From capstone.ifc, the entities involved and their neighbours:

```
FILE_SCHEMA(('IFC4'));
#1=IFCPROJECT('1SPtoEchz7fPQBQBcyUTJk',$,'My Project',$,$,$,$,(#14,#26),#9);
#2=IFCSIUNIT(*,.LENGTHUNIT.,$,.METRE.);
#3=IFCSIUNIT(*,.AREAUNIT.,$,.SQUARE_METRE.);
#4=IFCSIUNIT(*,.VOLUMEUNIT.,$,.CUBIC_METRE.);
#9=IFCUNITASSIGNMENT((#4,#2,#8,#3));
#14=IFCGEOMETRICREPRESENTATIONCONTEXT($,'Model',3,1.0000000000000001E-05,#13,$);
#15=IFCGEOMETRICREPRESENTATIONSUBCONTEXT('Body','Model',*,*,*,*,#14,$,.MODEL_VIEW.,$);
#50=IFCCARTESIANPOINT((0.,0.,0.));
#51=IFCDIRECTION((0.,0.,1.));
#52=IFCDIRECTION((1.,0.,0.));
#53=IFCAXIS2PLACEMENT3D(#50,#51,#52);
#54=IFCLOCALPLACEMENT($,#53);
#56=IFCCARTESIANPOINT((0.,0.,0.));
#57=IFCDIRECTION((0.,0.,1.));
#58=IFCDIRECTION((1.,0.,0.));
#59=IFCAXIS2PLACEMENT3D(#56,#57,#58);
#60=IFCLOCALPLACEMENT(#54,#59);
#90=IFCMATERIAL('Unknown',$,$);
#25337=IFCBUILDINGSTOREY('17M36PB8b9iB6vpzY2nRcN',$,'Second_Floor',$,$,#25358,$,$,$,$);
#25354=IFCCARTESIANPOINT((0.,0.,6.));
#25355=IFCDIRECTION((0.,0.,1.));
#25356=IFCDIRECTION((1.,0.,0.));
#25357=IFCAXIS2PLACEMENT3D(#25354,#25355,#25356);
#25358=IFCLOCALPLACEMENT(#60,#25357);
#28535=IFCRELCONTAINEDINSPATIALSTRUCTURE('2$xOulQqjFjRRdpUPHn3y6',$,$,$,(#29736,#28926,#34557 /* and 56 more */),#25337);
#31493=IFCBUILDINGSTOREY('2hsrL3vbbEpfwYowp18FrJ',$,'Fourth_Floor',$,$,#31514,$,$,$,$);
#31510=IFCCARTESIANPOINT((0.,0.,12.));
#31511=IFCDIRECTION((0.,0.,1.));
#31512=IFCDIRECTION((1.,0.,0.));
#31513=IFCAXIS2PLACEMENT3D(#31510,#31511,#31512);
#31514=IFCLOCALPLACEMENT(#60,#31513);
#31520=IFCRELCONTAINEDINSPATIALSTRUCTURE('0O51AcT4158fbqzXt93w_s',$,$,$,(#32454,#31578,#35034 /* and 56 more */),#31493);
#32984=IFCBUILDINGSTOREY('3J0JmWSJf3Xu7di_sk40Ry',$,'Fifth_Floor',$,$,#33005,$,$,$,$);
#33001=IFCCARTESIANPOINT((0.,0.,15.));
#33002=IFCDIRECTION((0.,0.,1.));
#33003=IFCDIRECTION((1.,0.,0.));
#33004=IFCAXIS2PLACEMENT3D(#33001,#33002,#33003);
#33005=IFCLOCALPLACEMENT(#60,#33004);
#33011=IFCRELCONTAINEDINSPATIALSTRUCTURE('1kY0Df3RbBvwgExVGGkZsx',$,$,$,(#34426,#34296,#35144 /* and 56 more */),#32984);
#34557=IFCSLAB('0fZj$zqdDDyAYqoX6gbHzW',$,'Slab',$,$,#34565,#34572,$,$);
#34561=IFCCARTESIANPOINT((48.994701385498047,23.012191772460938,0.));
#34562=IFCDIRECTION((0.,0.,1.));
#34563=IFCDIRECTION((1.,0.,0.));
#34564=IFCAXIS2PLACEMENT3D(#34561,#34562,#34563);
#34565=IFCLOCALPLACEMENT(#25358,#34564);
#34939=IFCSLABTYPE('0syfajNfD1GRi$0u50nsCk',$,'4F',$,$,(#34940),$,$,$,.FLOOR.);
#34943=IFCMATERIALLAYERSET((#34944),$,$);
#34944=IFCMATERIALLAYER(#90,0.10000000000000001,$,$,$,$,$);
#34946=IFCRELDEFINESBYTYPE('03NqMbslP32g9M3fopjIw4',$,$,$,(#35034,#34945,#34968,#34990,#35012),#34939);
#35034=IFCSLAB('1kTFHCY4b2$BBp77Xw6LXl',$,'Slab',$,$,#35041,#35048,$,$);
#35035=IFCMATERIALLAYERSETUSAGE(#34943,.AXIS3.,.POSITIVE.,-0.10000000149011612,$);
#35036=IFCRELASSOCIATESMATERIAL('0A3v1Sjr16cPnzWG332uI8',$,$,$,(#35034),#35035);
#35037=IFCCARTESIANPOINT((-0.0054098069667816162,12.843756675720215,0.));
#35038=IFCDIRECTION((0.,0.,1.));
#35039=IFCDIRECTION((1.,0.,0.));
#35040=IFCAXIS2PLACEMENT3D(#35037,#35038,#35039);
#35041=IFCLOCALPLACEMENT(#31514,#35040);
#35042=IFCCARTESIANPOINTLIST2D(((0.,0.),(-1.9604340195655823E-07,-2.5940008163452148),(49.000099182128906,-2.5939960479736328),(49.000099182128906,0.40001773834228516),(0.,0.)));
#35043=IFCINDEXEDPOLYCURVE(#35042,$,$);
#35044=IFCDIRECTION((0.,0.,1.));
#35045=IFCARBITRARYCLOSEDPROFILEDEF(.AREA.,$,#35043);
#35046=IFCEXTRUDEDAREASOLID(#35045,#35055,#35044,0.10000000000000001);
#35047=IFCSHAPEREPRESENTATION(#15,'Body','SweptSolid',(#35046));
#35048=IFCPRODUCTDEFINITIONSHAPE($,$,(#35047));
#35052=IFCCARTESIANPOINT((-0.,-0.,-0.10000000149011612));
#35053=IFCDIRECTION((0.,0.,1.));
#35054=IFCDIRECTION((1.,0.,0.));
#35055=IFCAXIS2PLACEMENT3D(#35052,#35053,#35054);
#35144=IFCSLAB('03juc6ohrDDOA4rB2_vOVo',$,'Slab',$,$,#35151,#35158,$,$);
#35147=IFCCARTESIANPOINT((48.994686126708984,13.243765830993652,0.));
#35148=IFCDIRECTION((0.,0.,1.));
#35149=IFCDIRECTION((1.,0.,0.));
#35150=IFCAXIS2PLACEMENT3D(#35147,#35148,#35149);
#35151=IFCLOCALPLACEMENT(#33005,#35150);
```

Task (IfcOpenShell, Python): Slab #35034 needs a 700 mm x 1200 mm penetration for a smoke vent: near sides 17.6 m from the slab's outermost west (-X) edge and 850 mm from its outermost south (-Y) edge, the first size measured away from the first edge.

```python
import numpy as np
import ifcopenshell
import ifcopenshell.api.feature
import ifcopenshell.api.geometry
import ifcopenshell.api.root
import ifcopenshell.geom
import ifcopenshell.util.placement
import ifcopenshell.util.representation
import ifcopenshell.util.shape
import ifcopenshell.util.unit

model = ifcopenshell.open("capstone.ifc")
unit_scale = ifcopenshell.util.unit.calculate_unit_scale(model)
settings = ifcopenshell.geom.settings()


def volume(element):
    """Net volume in cubic metres, openings subtracted."""
    shape = ifcopenshell.geom.create_shape(settings, element)
    return ifcopenshell.util.shape.get_volume(shape.geometry)


slab = model.by_guid("1kTFHCY4b2$BBp77Xw6LXl")
before = volume(slab)

# Extent in the slab's own axes, in metres. The edges named are its -X and -Y sides.
slab_shape = ifcopenshell.geom.create_shape(settings, slab)
vertices = ifcopenshell.util.shape.get_vertices(slab_shape.geometry)
x_min, y_min, bottom = vertices.min(axis=0)
top = vertices[:, 2].max()

opening = ifcopenshell.api.root.create_entity(model, ifc_class="IfcOpeningElement", name="Smoke vent opening", predefined_type="OPENING")
context = ifcopenshell.util.representation.get_context(model, "Model", "Body", "MODEL_VIEW")
width, depth = 0.7, 1.2
outline = [(0.0, 0.0), (width, 0.0), (width, depth), (0.0, depth), (0.0, 0.0)]
# Overshoot both faces by 50 mm so the cut is clean.
shape = ifcopenshell.api.geometry.add_slab_representation(
    model, context=context, depth=top - bottom + 0.1, polyline=outline
)
ifcopenshell.api.geometry.assign_representation(model, product=opening, representation=shape)

matrix = ifcopenshell.util.placement.get_local_placement(slab.ObjectPlacement)
matrix[:, 3] = matrix @ np.append(np.array([x_min + 17.6, y_min + 0.85, bottom - 0.05]) / unit_scale, 1.0)
ifcopenshell.api.geometry.edit_object_placement(model, product=opening, matrix=matrix, is_si=False)
ifcopenshell.api.feature.add_feature(model, feature=opening, element=slab)

after = volume(slab)

print(f"slab volume {before:.3f} -> {after:.3f} m3")

model.write("capstone_rev.ifc")
```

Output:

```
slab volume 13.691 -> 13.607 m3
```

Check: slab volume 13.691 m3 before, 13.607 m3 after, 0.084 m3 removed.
